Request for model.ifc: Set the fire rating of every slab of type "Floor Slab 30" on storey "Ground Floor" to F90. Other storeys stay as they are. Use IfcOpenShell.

First a look at what the model holds.

```python
import ifcopenshell
import ifcopenshell.util.element

model = ifcopenshell.open("model.ifc")
print(model.schema)
storey = next(s for s in model.by_type("IfcBuildingStorey") if s.Name == "Ground Floor")
slabs = [e for e in ifcopenshell.util.element.get_decomposition(storey) if e.is_a("IfcSlab")]
seen = {}
for e in slabs:
    element_type = ifcopenshell.util.element.get_type(e)
    key = (element_type.Name if element_type != e and element_type else None, ifcopenshell.util.element.get_pset(e, "Pset_SlabCommon", "FireRating"))
    seen[key] = seen.get(key, 0) + 1
for (name, value), count in sorted(seen.items(), key=str):
    print(count, "x", name, "|", value)
```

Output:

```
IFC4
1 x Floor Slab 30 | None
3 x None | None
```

```python
import ifcopenshell
import ifcopenshell.api.pset
import ifcopenshell.util.element

model = ifcopenshell.open("model.ifc")

storey = next(s for s in model.by_type("IfcBuildingStorey") if s.Name == "Ground Floor")
slabs = [e for e in ifcopenshell.util.element.get_decomposition(storey) if e.is_a("IfcSlab")]

count = 0
for e in slabs:
    element_type = ifcopenshell.util.element.get_type(e)
    if element_type in (None, e) or element_type.Name != "Floor Slab 30":
        continue
    # add_pset returns the element's existing set when there is one.
    pset = ifcopenshell.api.pset.add_pset(model, product=e, name="Pset_SlabCommon")
    ifcopenshell.api.pset.edit_pset(model, pset=pset, properties={"FireRating": "F90"})
    count += 1

print(count, "slabs updated")

model.write("model_edited.ifc")
```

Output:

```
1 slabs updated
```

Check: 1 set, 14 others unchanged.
